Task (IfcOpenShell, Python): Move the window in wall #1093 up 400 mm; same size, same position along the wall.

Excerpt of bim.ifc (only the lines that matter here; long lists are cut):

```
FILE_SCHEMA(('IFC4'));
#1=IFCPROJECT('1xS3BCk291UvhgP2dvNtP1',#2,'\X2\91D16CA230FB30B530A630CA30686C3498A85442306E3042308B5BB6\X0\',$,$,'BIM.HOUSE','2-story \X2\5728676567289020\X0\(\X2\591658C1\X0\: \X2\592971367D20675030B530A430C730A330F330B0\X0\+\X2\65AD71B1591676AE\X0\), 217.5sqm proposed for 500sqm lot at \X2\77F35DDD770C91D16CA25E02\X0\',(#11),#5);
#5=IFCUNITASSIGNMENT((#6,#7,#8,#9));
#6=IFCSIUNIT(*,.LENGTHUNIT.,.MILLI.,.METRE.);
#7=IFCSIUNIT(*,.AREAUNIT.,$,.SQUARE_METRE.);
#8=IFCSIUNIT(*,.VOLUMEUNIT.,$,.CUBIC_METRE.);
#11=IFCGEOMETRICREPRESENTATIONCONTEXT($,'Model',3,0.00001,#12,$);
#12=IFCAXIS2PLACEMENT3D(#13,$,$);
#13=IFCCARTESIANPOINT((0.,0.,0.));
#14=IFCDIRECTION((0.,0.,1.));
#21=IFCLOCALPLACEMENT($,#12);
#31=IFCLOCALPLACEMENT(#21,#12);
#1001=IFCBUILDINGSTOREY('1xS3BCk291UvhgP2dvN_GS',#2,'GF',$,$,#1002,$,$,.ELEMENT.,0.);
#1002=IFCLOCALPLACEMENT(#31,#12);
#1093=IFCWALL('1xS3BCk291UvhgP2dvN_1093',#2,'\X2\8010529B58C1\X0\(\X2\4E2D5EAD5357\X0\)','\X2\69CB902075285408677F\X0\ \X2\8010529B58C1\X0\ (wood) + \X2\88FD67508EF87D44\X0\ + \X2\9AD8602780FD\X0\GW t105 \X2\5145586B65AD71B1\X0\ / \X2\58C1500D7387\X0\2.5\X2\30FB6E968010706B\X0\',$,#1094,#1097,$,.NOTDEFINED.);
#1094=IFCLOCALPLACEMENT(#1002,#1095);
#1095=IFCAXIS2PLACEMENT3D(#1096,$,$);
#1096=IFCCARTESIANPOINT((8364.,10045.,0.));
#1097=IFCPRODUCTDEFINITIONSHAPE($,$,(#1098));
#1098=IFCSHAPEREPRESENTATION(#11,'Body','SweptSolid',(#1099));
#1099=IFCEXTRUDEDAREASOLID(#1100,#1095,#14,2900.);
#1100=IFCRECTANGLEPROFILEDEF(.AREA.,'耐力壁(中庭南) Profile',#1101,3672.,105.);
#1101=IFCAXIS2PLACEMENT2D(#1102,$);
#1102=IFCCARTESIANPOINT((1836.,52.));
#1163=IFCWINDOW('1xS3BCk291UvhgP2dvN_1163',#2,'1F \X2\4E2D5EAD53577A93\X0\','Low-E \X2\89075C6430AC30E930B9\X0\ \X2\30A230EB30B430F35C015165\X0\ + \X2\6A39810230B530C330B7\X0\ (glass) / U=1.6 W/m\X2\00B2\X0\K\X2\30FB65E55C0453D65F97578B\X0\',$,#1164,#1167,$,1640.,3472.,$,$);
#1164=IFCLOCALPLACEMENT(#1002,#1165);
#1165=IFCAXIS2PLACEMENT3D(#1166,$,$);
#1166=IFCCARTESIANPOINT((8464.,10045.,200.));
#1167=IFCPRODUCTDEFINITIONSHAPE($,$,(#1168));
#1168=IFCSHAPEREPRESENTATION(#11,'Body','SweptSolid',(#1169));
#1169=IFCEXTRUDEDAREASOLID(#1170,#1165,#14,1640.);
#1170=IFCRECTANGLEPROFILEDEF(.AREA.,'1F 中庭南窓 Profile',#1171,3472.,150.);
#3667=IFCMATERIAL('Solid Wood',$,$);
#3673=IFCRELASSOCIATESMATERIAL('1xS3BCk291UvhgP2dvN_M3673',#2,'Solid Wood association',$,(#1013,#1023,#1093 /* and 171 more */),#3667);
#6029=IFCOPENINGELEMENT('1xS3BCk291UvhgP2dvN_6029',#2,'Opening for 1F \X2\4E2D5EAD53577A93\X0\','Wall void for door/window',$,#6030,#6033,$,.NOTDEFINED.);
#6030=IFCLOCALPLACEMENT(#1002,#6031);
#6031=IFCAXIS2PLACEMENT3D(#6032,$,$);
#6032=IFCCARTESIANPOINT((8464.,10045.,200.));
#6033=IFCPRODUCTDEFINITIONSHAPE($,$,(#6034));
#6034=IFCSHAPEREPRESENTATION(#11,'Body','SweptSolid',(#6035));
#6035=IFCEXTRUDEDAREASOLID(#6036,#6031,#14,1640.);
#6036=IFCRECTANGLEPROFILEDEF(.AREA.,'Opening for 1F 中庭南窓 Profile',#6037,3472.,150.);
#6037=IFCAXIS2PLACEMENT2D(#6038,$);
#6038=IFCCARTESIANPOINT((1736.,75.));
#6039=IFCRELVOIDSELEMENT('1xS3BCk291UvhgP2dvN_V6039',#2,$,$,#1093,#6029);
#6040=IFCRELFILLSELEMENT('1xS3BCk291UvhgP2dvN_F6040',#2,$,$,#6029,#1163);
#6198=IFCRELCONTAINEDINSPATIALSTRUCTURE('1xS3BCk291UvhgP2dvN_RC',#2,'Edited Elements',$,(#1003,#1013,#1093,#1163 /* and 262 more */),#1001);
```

```python
import numpy as np
import ifcopenshell
import ifcopenshell.api.geometry
import ifcopenshell.util.placement
import ifcopenshell.util.unit

model = ifcopenshell.open("bim.ifc")
unit_scale = ifcopenshell.util.unit.calculate_unit_scale(model)

window = model.by_guid("1xS3BCk291UvhgP2dvN_1163")
opening = window.FillsVoids[0].RelatingOpeningElement
dz = 400.0

shift = np.array([0.0, 0.0, dz])
# The window is not placed relative to its opening, so move both.
for product in (opening, window):
    matrix = ifcopenshell.util.placement.get_local_placement(product.ObjectPlacement)
    matrix[:3, 3] += shift
    ifcopenshell.api.geometry.edit_object_placement(model, product=product, matrix=matrix, is_si=False)

print(f"moved by {dz * unit_scale:+.3f} m")

model.write("bim_updated.ifc")
```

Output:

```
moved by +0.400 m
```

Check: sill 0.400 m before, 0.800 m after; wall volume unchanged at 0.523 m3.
